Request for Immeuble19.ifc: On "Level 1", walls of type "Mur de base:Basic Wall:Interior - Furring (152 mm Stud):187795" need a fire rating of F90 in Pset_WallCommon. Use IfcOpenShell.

First a look at what the model holds.

```python
import ifcopenshell
import ifcopenshell.util.element

model = ifcopenshell.open("Immeuble19.ifc")
print(model.schema)
storey = next(s for s in model.by_type("IfcBuildingStorey") if s.Name == "Level 1")
walls = [e for e in ifcopenshell.util.element.get_decomposition(storey) if e.is_a("IfcWall")]
seen = {}
for e in walls:
    element_type = ifcopenshell.util.element.get_type(e)
    key = (element_type.Name if element_type != e and element_type else None, ifcopenshell.util.element.get_pset(e, "Pset_WallCommon", "FireRating"))
    seen[key] = seen.get(key, 0) + 1
for (name, value), count in sorted(seen.items(), key=str):
    print(count, "x", name, "|", value)
```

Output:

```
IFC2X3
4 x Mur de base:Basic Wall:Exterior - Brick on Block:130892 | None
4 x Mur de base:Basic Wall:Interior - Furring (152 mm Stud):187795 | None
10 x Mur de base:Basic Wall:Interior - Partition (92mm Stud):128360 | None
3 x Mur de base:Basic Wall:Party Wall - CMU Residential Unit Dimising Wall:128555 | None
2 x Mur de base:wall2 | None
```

```python
import ifcopenshell
import ifcopenshell.api.pset
import ifcopenshell.util.element

model = ifcopenshell.open("Immeuble19.ifc")

storey = next(s for s in model.by_type("IfcBuildingStorey") if s.Name == "Level 1")
walls = [e for e in ifcopenshell.util.element.get_decomposition(storey) if e.is_a("IfcWall")]

count = 0
for e in walls:
    element_type = ifcopenshell.util.element.get_type(e)
    if element_type in (None, e) or element_type.Name != "Mur de base:Basic Wall:Interior - Furring (152 mm Stud):187795":
        continue
    # add_pset returns the element's existing set when there is one.
    pset = ifcopenshell.api.pset.add_pset(model, product=e, name="Pset_WallCommon")
    ifcopenshell.api.pset.edit_pset(model, pset=pset, properties={"FireRating": "F90"})
    count += 1

print(count, "walls updated")

model.write("Immeuble19_rev.ifc")
```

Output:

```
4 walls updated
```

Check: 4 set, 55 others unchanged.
